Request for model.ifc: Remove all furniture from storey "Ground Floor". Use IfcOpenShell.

First a look at what the model holds.

```python
import ifcopenshell
import ifcopenshell.util.element

model = ifcopenshell.open("model.ifc")
print(model.schema)
storey = next(s for s in model.by_type("IfcBuildingStorey") if s.Name == "Ground Floor")
furniture = [e for e in ifcopenshell.util.element.get_decomposition(storey) if e.is_a("IfcFurnishingElement")]
seen = {}
for e in furniture:
    element_type = ifcopenshell.util.element.get_type(e)
    name = element_type.Name if element_type not in (None, e) else None
    seen[name] = seen.get(name, 0) + 1
for name, count in sorted(seen.items(), key=str):
    print(count, "x", name)
```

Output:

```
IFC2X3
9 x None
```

```python
import ifcopenshell
import ifcopenshell.api.root
import ifcopenshell.util.element

model = ifcopenshell.open("model.ifc")

storey = next(s for s in model.by_type("IfcBuildingStorey") if s.Name == "Ground Floor")
furniture = [e for e in ifcopenshell.util.element.get_decomposition(storey) if e.is_a("IfcFurnishingElement")]

for e in furniture:
    ifcopenshell.api.root.remove_product(model, product=e)
print(len(furniture), "removed")

model.write("model-out.ifc")
```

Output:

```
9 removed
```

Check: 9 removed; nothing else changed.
